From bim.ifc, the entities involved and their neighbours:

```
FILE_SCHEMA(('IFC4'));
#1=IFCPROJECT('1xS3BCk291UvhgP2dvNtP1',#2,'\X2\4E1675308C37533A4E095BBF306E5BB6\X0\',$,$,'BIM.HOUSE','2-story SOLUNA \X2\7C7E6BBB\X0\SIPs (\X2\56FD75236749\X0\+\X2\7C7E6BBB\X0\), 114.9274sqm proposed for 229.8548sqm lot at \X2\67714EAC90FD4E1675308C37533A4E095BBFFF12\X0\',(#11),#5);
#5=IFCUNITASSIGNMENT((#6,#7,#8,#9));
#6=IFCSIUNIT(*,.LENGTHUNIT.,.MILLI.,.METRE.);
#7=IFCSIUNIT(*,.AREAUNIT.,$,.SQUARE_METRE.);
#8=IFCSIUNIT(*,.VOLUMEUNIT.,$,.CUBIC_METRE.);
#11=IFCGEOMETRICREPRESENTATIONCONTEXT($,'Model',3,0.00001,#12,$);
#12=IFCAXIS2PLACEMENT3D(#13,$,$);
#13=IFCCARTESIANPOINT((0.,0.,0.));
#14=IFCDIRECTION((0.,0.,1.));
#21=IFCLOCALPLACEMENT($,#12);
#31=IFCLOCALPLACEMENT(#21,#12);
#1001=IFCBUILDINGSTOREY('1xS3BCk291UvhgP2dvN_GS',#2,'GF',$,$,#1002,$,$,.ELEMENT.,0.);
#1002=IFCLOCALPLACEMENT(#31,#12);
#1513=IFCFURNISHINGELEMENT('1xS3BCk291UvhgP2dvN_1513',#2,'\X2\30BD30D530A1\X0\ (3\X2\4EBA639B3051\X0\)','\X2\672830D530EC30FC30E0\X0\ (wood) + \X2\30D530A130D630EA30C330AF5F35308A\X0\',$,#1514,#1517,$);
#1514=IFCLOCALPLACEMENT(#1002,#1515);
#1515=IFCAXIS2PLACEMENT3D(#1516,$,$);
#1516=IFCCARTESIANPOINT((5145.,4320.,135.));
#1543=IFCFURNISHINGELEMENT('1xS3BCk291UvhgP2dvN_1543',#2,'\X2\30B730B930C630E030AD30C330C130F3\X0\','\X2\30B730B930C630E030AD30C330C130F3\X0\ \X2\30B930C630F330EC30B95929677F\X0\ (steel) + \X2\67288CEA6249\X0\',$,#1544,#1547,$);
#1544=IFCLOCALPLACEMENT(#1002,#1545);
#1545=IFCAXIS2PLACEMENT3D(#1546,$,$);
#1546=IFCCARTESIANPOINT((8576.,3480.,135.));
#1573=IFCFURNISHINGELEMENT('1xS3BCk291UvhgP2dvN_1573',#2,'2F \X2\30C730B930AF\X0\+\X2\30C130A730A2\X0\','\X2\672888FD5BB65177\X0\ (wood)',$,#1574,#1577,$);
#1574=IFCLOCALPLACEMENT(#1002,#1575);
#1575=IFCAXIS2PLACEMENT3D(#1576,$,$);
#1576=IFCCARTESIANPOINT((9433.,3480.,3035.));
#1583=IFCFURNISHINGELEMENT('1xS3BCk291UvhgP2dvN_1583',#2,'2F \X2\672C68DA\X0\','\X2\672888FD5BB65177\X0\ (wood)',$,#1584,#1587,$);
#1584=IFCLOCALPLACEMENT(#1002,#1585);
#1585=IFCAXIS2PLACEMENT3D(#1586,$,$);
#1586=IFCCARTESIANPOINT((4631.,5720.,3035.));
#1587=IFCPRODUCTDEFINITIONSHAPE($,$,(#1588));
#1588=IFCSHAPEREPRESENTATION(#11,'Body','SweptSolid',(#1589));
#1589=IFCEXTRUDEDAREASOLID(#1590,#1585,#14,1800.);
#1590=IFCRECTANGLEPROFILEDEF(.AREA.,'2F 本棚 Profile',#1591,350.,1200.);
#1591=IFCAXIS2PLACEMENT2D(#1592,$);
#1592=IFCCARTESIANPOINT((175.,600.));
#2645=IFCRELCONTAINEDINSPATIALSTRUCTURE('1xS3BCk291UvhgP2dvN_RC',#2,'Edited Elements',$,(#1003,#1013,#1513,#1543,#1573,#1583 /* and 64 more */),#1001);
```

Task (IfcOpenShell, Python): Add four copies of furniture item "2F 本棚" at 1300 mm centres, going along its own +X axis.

```python
import ifcopenshell
import ifcopenshell.api.geometry
import ifcopenshell.api.root
import ifcopenshell.util.element
import ifcopenshell.util.placement
import ifcopenshell.util.unit

model = ifcopenshell.open("bim.ifc")
unit_scale = ifcopenshell.util.unit.calculate_unit_scale(model)


def reuse_history(source, copy):
    """copy_class also copies each property set's owner history, people and application; keep the originals."""
    for rel in copy.IsDefinedBy:
        if rel.is_a("IfcRelDefinesByProperties") and (history := rel.RelatingPropertyDefinition.OwnerHistory):
            rel.RelatingPropertyDefinition.OwnerHistory = source.OwnerHistory
            ifcopenshell.util.element.remove_deep2(model, history)


source = model.by_guid("1xS3BCk291UvhgP2dvN_1583")
base = ifcopenshell.util.placement.get_local_placement(source.ObjectPlacement)
step = base[:3, 0] * 1.3 / unit_scale

for i in range(1, 5):
    copy = ifcopenshell.api.root.copy_class(model, product=source)
    copy.Representation = ifcopenshell.util.element.copy_deep(
        model, source.Representation, exclude=["IfcGeometricRepresentationContext", "IfcRepresentationMap"]
    )
    reuse_history(source, copy)
    matrix = base.copy()
    matrix[:3, 3] += i * step
    print("added at", matrix[:3, 3].round(3) + 0.0)
    ifcopenshell.api.geometry.edit_object_placement(model, product=copy, matrix=matrix, is_si=False)

model.write("bim_v2.ifc")
```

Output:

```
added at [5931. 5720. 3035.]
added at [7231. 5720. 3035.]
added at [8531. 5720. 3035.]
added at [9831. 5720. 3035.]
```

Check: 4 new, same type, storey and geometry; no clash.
